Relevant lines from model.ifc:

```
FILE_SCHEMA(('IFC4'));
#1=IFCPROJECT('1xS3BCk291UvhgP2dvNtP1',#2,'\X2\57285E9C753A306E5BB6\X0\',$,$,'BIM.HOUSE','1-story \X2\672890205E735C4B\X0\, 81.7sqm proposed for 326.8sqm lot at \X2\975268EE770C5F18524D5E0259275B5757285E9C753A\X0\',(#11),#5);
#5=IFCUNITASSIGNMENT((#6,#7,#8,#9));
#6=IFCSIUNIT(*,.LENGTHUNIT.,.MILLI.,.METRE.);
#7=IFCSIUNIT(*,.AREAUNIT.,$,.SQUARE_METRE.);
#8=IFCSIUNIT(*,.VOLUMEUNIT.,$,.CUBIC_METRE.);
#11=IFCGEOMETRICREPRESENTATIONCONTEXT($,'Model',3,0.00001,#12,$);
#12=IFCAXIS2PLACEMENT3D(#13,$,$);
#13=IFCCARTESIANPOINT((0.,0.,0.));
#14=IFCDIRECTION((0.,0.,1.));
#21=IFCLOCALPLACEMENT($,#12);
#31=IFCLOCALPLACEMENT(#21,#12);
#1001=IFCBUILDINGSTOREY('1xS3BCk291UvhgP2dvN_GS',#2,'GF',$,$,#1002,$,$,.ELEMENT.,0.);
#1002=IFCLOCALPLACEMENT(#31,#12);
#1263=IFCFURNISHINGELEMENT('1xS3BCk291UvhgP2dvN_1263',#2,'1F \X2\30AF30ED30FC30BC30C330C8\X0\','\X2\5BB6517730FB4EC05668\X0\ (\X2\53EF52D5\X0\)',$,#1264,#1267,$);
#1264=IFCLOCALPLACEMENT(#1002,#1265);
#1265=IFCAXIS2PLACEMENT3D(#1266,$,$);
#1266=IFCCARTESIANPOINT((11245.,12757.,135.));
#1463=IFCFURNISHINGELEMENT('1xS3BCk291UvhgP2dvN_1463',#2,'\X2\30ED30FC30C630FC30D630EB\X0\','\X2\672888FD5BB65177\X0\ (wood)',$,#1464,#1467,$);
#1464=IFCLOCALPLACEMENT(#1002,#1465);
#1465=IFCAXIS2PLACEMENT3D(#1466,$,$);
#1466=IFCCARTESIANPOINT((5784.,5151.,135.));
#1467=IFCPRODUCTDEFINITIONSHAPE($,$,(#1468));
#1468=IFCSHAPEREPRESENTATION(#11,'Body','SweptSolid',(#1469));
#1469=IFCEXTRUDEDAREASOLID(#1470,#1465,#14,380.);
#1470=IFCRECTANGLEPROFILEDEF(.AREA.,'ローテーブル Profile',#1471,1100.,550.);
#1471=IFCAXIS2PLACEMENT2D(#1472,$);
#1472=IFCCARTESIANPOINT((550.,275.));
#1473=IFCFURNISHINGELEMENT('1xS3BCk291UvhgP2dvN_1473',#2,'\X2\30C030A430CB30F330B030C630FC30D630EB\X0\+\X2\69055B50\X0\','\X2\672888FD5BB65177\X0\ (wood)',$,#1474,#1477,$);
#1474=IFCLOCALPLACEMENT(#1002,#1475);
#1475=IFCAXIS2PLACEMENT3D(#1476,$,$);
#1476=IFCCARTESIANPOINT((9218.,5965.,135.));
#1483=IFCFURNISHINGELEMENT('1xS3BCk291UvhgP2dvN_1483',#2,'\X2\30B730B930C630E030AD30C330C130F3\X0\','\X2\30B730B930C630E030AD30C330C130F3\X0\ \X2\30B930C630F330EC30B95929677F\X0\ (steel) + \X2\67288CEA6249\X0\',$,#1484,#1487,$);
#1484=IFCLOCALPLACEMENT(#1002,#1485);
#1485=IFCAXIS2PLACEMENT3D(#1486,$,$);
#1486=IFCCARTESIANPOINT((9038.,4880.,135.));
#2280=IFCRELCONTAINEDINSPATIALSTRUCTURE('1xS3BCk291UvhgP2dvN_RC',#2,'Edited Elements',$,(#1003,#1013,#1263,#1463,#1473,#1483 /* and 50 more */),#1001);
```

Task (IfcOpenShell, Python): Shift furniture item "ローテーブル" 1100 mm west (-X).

```python
import ifcopenshell
import ifcopenshell.api.geometry
import ifcopenshell.util.placement
import ifcopenshell.util.unit

model = ifcopenshell.open("model.ifc")
unit_scale = ifcopenshell.util.unit.calculate_unit_scale(model)

item = model.by_guid("1xS3BCk291UvhgP2dvN_1463")
matrix = ifcopenshell.util.placement.get_local_placement(item.ObjectPlacement)
matrix[0, 3] -= 1.1 / unit_scale
ifcopenshell.api.geometry.edit_object_placement(model, product=item, matrix=matrix, is_si=False)

print(ifcopenshell.util.placement.get_local_placement(item.ObjectPlacement).round(3) + 0.0)

model.write("model_v2.ifc")
```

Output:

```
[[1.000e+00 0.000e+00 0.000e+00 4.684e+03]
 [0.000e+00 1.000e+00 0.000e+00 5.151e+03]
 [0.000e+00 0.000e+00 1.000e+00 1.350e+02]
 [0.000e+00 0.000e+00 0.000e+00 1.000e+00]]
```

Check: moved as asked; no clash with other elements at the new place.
